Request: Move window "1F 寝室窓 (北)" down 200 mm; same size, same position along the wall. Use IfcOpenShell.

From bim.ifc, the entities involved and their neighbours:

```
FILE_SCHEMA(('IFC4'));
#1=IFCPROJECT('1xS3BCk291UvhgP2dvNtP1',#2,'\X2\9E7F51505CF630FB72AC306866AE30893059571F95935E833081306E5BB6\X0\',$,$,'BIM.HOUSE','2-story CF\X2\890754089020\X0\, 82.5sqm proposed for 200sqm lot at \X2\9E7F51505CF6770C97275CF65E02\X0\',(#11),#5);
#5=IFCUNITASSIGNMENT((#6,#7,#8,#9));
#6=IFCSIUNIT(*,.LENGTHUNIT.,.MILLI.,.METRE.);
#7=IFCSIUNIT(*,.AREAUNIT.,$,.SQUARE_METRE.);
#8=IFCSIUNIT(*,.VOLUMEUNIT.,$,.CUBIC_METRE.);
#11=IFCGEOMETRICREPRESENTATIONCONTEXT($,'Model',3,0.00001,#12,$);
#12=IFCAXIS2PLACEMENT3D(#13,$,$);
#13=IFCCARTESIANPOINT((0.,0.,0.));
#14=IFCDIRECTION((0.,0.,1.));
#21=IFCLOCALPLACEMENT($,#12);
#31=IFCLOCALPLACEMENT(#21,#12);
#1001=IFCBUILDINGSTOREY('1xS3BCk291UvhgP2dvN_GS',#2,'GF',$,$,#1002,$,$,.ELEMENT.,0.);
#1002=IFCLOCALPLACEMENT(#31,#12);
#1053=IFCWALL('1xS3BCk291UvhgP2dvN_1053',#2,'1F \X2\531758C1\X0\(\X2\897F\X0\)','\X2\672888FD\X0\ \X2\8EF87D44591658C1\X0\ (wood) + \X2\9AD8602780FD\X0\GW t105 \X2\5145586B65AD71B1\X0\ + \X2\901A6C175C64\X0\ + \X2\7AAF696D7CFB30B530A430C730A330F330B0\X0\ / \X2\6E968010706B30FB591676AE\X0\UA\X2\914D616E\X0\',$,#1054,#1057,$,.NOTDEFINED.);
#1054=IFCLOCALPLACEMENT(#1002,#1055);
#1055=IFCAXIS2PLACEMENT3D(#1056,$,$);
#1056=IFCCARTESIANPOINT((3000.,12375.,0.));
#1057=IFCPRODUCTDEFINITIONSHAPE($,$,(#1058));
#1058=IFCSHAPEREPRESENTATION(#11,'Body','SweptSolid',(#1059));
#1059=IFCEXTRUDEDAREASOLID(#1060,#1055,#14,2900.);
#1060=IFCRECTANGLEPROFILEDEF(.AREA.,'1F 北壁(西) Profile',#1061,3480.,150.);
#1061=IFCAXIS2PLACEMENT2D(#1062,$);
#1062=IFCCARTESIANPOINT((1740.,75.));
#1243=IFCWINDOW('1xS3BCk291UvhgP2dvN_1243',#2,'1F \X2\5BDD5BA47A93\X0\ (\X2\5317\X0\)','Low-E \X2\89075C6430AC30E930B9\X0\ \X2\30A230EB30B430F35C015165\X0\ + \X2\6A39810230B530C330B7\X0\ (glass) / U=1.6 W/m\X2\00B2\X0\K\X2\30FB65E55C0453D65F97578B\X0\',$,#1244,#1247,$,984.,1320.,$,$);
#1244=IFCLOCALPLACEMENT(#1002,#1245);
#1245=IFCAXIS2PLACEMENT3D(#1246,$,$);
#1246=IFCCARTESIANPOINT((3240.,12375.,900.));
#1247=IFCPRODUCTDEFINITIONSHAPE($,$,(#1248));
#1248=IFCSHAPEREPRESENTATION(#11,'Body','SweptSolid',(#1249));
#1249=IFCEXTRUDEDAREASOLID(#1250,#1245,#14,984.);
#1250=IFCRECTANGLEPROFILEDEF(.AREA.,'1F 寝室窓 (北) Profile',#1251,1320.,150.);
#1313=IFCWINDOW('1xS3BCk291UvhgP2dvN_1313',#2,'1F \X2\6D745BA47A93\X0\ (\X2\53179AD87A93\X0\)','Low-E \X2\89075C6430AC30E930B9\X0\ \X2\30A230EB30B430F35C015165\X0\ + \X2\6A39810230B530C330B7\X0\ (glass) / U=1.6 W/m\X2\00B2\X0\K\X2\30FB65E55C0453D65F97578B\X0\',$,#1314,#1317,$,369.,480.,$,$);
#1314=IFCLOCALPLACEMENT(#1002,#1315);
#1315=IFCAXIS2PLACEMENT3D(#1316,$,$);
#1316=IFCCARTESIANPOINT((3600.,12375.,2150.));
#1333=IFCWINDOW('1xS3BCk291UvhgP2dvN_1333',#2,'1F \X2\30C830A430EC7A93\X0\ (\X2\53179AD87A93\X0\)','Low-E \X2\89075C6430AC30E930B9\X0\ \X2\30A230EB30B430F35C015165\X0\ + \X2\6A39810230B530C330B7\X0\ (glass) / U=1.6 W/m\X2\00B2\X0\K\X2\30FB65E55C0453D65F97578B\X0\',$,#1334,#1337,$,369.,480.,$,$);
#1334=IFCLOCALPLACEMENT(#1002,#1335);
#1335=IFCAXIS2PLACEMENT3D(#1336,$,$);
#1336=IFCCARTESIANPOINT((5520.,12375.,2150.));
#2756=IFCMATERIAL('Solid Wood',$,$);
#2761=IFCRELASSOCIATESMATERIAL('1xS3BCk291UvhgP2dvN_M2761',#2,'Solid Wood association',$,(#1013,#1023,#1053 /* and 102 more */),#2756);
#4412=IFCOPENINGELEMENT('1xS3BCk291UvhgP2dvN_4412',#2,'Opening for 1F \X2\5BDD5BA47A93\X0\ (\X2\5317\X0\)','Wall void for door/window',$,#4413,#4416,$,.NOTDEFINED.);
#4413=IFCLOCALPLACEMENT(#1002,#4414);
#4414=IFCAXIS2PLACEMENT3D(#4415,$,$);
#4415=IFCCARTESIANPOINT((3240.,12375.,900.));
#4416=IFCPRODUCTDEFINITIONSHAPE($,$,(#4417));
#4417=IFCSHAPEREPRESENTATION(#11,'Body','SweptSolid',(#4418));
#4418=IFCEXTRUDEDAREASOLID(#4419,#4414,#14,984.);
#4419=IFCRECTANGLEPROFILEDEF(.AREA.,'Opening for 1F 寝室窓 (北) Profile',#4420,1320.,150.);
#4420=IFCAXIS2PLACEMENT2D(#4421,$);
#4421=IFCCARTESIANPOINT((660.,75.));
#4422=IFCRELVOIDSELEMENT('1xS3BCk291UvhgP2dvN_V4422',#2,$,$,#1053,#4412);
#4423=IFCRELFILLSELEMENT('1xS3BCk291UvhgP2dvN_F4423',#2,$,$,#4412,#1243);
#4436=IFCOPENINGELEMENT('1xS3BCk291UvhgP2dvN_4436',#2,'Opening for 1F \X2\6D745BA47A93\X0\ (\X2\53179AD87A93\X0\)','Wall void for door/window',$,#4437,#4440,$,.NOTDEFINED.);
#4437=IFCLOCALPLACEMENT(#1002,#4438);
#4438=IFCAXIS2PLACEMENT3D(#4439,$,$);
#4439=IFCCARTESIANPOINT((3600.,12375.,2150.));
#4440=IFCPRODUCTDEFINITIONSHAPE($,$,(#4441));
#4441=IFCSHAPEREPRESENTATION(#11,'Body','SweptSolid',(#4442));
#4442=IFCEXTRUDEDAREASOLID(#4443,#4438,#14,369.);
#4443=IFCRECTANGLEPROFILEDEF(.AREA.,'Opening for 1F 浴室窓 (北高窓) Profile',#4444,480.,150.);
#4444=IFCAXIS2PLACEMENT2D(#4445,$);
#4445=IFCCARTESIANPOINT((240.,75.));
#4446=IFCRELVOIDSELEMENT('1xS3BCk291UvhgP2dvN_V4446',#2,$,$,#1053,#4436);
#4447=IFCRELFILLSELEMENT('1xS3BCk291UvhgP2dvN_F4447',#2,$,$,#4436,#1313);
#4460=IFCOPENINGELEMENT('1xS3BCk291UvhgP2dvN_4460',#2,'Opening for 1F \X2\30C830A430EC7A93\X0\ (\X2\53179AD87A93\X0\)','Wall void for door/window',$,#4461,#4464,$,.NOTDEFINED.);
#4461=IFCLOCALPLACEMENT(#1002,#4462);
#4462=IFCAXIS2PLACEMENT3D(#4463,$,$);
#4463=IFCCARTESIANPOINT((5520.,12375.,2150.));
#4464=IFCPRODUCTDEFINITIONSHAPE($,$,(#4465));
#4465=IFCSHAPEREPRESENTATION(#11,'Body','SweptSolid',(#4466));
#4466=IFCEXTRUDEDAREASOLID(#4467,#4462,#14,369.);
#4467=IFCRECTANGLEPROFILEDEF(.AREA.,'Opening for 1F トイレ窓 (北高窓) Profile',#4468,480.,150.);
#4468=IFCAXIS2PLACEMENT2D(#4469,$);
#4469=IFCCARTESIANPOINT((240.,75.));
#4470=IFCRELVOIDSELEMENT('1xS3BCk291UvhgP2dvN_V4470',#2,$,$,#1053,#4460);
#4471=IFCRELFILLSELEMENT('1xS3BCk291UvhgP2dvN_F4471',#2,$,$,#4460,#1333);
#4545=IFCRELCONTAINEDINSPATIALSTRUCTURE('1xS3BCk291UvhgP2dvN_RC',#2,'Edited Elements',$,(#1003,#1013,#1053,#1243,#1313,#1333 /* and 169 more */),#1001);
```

```python
import numpy as np
import ifcopenshell
import ifcopenshell.api.geometry
import ifcopenshell.util.placement
import ifcopenshell.util.unit

model = ifcopenshell.open("bim.ifc")
unit_scale = ifcopenshell.util.unit.calculate_unit_scale(model)

window = model.by_guid("1xS3BCk291UvhgP2dvN_1243")
opening = window.FillsVoids[0].RelatingOpeningElement
dz = -0.2 / unit_scale

shift = np.array([0.0, 0.0, dz])
# The window is not placed relative to its opening, so move both.
for product in (opening, window):
    matrix = ifcopenshell.util.placement.get_local_placement(product.ObjectPlacement)
    matrix[:3, 3] += shift
    ifcopenshell.api.geometry.edit_object_placement(model, product=product, matrix=matrix, is_si=False)

print(f"moved by {dz * unit_scale:+.3f} m")

model.write("bim-out.ifc")
```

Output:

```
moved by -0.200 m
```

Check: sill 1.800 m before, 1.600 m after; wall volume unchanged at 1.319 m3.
